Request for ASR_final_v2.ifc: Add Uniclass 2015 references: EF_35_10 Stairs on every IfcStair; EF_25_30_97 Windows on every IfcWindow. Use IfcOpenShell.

First a look at what the model holds.

```python
import ifcopenshell

model = ifcopenshell.open("ASR_final_v2.ifc")
print(model.schema)
print("classifications:", [c.Name for c in model.by_type("IfcClassification")])
for ifc_class in ("IfcDoor", "IfcRoof", "IfcStair", "IfcWall", "IfcWindow"):
    print(ifc_class, len(model.by_type(ifc_class)))
```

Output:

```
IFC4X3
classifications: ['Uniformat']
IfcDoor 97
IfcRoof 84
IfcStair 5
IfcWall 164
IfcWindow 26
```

```python
import ifcopenshell
import ifcopenshell.api.classification

model = ifcopenshell.open("ASR_final_v2.ifc")

system = ifcopenshell.api.classification.add_classification(model, classification="Uniclass 2015")

codes = {
    "IfcStair": ("EF_35_10", "Stairs"),
    "IfcWindow": ("EF_25_30_97", "Windows"),
}
for ifc_class, (code, name) in codes.items():
    products = model.by_type(ifc_class)
    ifcopenshell.api.classification.add_reference(
        model, products=products, classification=system, identification=code, name=name
    )
    print(code, len(products))

model.write("ASR_final_v2_rev.ifc")
```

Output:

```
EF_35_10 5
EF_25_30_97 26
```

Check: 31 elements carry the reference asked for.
